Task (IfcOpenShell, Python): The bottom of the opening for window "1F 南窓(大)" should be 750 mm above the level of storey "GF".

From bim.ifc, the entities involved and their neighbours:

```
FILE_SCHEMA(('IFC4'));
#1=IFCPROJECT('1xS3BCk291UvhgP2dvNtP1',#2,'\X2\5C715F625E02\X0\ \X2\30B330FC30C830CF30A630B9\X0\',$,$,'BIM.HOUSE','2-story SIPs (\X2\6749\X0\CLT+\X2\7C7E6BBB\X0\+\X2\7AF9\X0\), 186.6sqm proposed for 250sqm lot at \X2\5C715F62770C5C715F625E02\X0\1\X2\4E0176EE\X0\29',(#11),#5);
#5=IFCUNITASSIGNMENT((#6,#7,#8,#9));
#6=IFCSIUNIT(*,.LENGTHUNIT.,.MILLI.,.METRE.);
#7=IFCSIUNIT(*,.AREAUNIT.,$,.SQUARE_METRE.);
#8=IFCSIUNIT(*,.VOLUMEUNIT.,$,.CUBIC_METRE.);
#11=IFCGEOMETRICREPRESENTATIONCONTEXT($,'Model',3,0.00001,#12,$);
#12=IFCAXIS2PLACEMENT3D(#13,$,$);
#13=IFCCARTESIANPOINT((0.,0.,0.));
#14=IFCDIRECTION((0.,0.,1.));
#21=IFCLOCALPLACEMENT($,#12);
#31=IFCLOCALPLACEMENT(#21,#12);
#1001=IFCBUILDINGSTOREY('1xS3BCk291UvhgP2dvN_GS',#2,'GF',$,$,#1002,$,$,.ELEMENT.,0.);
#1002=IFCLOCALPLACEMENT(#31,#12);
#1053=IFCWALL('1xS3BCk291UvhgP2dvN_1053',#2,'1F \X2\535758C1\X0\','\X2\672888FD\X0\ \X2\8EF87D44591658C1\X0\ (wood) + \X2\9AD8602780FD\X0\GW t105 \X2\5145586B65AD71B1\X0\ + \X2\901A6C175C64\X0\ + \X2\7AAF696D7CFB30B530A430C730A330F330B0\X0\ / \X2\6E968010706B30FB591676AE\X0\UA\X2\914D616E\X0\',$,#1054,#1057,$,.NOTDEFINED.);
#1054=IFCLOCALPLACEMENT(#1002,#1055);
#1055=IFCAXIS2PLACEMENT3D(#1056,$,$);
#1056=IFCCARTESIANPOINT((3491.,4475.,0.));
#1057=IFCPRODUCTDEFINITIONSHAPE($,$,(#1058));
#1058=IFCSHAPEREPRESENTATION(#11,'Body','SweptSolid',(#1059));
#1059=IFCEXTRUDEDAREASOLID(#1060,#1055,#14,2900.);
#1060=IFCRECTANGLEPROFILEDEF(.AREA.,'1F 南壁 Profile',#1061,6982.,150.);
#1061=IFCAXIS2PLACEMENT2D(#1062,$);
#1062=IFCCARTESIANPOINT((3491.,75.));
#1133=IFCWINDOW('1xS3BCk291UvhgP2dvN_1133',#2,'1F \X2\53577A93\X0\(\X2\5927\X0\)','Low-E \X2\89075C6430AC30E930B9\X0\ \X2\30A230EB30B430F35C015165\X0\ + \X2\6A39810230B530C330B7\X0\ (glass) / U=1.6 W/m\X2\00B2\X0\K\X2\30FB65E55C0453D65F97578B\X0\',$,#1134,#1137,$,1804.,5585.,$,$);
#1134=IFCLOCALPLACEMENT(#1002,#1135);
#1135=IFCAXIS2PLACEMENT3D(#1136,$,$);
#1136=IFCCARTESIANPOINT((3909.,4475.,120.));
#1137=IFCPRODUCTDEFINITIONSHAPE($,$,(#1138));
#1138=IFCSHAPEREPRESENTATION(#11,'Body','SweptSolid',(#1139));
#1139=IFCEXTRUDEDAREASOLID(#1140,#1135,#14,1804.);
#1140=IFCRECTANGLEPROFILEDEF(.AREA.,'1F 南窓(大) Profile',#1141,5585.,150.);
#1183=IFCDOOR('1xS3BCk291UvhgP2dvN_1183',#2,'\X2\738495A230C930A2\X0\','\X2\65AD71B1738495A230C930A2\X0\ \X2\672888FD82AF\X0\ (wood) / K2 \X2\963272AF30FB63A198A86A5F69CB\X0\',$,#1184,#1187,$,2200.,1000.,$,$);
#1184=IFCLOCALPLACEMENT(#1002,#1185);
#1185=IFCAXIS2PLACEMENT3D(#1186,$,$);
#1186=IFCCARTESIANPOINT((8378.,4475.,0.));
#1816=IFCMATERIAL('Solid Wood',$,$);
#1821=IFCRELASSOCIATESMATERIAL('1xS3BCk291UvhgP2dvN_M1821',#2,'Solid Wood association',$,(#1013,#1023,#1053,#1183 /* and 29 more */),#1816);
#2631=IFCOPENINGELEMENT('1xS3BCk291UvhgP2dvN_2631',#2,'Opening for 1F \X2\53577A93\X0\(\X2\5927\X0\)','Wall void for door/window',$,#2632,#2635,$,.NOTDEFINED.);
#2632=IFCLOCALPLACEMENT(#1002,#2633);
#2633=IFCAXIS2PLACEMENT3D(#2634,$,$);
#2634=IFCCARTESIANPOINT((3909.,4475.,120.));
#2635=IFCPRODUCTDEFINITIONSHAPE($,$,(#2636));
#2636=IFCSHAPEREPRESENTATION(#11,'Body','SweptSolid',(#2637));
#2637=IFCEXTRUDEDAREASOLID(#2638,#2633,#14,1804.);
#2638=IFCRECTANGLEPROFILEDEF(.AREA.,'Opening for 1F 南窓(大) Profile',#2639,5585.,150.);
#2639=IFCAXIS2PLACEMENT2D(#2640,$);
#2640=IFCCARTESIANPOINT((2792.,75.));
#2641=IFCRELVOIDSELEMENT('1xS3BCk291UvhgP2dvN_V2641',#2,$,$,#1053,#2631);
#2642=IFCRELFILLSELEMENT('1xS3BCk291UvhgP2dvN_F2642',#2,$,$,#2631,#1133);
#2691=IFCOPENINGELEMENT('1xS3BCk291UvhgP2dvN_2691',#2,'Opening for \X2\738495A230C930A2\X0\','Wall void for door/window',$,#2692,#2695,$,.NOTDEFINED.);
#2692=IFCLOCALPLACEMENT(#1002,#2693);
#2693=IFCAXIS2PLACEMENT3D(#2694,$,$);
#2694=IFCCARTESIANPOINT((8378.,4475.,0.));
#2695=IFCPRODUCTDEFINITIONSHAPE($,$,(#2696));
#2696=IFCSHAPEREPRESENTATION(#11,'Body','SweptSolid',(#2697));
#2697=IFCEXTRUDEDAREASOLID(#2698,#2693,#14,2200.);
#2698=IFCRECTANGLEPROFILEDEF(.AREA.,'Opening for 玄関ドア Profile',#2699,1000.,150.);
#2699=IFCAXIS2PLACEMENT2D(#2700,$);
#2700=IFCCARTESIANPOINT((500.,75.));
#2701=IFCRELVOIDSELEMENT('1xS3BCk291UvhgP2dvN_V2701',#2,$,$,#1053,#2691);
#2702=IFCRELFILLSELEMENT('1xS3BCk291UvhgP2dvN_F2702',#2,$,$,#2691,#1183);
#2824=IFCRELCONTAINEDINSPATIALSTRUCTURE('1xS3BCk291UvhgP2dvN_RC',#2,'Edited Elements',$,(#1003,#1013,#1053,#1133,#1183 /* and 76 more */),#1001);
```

```python
import numpy as np
import ifcopenshell
import ifcopenshell.api.geometry
import ifcopenshell.geom
import ifcopenshell.util.element
import ifcopenshell.util.placement
import ifcopenshell.util.shape
import ifcopenshell.util.unit

model = ifcopenshell.open("bim.ifc")
unit_scale = ifcopenshell.util.unit.calculate_unit_scale(model)

window = model.by_id(1133)
opening = window.FillsVoids[0].RelatingOpeningElement
storey = ifcopenshell.util.element.get_container(window, ifc_class="IfcBuildingStorey")
level = ifcopenshell.util.placement.get_local_placement(storey.ObjectPlacement)[2, 3]

# The opening's origin need not be at the sill, so measure its lowest point.
shape = ifcopenshell.geom.create_shape(ifcopenshell.geom.settings(), opening)
bottom = ifcopenshell.util.shape.get_shape_bottom_elevation(shape, shape.geometry) / unit_scale
dz = level + 750.0 - bottom

shift = np.array([0.0, 0.0, dz])
# The window is not placed relative to its opening, so move both.
for product in (opening, window):
    matrix = ifcopenshell.util.placement.get_local_placement(product.ObjectPlacement)
    matrix[:3, 3] += shift
    ifcopenshell.api.geometry.edit_object_placement(model, product=product, matrix=matrix, is_si=False)

print(f"moved by {dz * unit_scale:+.3f} m")

model.write("bim_edited.ifc")
```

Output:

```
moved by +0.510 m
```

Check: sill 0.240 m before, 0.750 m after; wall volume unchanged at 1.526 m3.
